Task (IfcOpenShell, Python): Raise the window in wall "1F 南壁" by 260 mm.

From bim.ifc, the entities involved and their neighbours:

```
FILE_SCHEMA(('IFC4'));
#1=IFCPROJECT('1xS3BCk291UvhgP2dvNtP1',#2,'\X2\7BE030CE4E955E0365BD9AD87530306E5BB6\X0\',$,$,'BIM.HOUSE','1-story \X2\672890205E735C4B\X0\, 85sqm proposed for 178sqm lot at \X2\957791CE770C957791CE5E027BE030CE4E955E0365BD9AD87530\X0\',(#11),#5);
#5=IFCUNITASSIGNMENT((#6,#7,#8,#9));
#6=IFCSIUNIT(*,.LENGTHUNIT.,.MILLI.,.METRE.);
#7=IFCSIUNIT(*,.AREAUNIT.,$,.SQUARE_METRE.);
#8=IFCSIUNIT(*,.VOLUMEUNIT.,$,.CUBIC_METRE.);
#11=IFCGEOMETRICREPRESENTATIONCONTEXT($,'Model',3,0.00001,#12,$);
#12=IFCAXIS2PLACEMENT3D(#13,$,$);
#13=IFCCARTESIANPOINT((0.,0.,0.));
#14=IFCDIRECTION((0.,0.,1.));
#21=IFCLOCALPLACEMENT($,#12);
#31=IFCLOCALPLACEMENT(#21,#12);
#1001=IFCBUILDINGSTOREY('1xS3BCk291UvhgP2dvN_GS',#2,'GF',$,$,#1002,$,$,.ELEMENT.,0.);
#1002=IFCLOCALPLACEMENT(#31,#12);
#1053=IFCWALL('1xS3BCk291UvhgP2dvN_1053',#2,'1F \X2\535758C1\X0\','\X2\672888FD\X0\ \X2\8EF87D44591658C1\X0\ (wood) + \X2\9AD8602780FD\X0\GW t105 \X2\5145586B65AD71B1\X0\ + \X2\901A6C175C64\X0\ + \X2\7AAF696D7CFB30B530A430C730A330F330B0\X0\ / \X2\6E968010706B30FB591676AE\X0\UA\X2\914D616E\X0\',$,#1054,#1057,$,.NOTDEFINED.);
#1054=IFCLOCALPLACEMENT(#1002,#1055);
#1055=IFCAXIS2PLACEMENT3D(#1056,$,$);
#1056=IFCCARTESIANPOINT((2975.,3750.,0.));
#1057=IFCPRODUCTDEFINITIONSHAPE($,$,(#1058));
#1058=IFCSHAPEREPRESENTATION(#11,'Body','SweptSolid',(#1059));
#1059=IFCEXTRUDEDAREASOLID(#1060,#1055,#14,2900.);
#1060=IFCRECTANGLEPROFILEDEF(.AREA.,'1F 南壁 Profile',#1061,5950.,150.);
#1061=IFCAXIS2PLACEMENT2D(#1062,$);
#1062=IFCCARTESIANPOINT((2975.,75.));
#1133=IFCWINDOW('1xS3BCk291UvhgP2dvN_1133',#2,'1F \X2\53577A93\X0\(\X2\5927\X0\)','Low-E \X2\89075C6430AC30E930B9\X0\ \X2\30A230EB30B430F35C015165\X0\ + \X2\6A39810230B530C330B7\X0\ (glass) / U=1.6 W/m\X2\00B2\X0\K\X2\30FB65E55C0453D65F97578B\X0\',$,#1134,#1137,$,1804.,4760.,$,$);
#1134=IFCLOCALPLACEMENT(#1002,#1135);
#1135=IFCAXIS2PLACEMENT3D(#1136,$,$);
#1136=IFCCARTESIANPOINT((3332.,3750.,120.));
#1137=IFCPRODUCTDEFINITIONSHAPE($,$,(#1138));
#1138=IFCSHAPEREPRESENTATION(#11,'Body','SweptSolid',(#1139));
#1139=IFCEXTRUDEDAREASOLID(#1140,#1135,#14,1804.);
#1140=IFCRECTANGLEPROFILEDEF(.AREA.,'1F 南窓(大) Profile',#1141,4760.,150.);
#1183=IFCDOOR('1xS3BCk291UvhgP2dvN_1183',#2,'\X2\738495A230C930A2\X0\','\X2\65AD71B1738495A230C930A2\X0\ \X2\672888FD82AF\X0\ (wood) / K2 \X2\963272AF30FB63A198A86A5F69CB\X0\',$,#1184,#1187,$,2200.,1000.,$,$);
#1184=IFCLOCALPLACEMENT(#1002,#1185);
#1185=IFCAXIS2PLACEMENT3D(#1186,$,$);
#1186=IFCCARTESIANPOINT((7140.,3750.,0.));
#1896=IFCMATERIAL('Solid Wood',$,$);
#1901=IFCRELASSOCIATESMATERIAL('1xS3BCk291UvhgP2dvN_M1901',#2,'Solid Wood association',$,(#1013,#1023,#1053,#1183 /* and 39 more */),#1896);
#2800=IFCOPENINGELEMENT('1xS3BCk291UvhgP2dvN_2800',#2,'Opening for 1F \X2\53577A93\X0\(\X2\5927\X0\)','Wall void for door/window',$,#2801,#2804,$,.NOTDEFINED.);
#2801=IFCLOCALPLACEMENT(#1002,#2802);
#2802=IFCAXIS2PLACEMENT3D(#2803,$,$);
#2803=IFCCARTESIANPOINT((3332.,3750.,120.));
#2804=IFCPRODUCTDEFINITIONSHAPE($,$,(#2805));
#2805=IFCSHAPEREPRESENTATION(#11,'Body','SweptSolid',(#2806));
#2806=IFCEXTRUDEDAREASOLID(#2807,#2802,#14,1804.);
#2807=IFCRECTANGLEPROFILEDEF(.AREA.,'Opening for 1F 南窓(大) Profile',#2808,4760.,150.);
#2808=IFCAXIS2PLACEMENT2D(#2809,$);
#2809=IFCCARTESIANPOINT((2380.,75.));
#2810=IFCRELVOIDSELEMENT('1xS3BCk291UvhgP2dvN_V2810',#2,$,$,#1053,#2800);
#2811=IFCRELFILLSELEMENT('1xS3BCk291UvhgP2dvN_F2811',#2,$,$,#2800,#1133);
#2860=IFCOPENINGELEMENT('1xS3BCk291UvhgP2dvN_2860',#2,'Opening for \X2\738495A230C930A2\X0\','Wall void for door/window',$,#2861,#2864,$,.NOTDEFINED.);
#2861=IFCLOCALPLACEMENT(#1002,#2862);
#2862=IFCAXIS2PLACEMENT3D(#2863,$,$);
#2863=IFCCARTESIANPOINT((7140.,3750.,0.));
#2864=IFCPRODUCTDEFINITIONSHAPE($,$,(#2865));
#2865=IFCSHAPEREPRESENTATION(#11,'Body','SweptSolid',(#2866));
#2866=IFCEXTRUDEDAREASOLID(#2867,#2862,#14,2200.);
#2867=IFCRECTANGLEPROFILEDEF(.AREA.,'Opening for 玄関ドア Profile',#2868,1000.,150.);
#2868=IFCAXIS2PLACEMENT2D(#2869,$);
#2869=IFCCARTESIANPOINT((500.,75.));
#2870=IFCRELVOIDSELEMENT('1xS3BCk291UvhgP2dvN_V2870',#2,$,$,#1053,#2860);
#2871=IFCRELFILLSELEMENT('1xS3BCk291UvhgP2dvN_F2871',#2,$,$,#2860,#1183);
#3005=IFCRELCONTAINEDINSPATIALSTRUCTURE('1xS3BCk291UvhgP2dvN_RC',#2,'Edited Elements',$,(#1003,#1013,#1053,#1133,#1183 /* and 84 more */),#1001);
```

```python
import numpy as np
import ifcopenshell
import ifcopenshell.api.geometry
import ifcopenshell.util.placement
import ifcopenshell.util.unit

model = ifcopenshell.open("bim.ifc")
unit_scale = ifcopenshell.util.unit.calculate_unit_scale(model)

window = model.by_guid("1xS3BCk291UvhgP2dvN_1133")
opening = window.FillsVoids[0].RelatingOpeningElement
dz = 260.0

shift = np.array([0.0, 0.0, dz])
# The window is not placed relative to its opening, so move both.
for product in (opening, window):
    matrix = ifcopenshell.util.placement.get_local_placement(product.ObjectPlacement)
    matrix[:3, 3] += shift
    ifcopenshell.api.geometry.edit_object_placement(model, product=product, matrix=matrix, is_si=False)

print(f"moved by {dz * unit_scale:+.3f} m")

model.write("bim_updated.ifc")
```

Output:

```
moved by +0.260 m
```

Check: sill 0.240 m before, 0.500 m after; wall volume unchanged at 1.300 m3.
